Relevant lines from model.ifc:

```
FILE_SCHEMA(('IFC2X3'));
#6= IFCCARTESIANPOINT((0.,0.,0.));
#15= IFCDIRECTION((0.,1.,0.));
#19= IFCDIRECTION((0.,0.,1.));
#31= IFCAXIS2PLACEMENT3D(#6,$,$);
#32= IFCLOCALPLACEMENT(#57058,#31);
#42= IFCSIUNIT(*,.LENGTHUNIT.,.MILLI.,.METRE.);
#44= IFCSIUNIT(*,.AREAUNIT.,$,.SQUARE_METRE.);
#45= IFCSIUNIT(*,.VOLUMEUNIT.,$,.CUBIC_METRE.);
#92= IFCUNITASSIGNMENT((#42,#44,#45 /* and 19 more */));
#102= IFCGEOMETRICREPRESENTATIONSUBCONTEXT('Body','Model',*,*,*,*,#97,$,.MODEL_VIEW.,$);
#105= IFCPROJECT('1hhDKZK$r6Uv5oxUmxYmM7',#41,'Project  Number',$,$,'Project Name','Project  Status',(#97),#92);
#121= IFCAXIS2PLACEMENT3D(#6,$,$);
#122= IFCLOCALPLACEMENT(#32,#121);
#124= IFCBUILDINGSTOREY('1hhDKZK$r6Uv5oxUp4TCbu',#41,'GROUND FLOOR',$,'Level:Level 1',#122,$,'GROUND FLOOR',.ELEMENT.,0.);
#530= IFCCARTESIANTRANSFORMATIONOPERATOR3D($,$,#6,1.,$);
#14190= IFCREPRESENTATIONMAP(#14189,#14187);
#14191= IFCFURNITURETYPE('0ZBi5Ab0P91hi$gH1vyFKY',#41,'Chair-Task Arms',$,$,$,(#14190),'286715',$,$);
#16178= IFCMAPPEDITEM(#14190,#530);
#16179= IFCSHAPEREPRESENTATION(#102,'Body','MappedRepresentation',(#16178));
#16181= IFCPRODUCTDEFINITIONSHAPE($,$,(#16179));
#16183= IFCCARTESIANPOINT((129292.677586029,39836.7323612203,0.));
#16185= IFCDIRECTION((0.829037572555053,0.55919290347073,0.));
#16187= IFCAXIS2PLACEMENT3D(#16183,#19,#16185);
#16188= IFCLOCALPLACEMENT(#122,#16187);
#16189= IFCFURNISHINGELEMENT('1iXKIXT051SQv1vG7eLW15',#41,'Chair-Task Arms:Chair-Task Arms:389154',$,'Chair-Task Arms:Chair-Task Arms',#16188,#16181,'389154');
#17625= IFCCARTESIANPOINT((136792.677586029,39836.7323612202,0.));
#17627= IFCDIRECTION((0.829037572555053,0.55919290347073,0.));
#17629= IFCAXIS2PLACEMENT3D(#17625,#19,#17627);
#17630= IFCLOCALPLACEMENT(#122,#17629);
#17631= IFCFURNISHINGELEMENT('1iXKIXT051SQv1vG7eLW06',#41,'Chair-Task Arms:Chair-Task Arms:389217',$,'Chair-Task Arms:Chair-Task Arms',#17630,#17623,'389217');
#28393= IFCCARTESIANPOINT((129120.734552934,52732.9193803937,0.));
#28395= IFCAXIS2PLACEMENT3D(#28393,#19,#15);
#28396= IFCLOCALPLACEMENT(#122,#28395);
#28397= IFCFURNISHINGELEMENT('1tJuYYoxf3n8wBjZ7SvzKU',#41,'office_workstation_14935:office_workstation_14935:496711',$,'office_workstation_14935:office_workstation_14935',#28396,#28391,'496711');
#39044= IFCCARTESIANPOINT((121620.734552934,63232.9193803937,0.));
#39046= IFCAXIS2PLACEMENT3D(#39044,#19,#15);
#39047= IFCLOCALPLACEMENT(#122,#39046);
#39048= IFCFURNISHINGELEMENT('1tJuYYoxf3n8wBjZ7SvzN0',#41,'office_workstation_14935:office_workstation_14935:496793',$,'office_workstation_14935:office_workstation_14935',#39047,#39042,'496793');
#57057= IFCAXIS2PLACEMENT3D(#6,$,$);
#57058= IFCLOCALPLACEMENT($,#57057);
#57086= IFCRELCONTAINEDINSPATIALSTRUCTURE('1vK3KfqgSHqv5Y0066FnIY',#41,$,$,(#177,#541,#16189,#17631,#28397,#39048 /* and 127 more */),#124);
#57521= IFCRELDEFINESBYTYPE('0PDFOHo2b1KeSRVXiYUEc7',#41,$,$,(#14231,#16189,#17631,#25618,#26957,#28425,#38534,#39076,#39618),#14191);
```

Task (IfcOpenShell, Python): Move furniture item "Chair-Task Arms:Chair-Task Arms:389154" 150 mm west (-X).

```python
import ifcopenshell
import ifcopenshell.api.geometry
import ifcopenshell.util.placement

model = ifcopenshell.open("model.ifc")

item = model.by_guid("1iXKIXT051SQv1vG7eLW15")
matrix = ifcopenshell.util.placement.get_local_placement(item.ObjectPlacement)
matrix[0, 3] -= 150.0
ifcopenshell.api.geometry.edit_object_placement(model, product=item, matrix=matrix, is_si=False)

print(ifcopenshell.util.placement.get_local_placement(item.ObjectPlacement).round(3) + 0.0)

model.write("model_edited.ifc")
```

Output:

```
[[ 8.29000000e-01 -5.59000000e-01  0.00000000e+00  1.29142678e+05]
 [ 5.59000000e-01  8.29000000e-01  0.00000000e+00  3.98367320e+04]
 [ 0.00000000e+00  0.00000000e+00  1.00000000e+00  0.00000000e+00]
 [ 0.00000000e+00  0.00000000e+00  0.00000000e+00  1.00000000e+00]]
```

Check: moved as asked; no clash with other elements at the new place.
